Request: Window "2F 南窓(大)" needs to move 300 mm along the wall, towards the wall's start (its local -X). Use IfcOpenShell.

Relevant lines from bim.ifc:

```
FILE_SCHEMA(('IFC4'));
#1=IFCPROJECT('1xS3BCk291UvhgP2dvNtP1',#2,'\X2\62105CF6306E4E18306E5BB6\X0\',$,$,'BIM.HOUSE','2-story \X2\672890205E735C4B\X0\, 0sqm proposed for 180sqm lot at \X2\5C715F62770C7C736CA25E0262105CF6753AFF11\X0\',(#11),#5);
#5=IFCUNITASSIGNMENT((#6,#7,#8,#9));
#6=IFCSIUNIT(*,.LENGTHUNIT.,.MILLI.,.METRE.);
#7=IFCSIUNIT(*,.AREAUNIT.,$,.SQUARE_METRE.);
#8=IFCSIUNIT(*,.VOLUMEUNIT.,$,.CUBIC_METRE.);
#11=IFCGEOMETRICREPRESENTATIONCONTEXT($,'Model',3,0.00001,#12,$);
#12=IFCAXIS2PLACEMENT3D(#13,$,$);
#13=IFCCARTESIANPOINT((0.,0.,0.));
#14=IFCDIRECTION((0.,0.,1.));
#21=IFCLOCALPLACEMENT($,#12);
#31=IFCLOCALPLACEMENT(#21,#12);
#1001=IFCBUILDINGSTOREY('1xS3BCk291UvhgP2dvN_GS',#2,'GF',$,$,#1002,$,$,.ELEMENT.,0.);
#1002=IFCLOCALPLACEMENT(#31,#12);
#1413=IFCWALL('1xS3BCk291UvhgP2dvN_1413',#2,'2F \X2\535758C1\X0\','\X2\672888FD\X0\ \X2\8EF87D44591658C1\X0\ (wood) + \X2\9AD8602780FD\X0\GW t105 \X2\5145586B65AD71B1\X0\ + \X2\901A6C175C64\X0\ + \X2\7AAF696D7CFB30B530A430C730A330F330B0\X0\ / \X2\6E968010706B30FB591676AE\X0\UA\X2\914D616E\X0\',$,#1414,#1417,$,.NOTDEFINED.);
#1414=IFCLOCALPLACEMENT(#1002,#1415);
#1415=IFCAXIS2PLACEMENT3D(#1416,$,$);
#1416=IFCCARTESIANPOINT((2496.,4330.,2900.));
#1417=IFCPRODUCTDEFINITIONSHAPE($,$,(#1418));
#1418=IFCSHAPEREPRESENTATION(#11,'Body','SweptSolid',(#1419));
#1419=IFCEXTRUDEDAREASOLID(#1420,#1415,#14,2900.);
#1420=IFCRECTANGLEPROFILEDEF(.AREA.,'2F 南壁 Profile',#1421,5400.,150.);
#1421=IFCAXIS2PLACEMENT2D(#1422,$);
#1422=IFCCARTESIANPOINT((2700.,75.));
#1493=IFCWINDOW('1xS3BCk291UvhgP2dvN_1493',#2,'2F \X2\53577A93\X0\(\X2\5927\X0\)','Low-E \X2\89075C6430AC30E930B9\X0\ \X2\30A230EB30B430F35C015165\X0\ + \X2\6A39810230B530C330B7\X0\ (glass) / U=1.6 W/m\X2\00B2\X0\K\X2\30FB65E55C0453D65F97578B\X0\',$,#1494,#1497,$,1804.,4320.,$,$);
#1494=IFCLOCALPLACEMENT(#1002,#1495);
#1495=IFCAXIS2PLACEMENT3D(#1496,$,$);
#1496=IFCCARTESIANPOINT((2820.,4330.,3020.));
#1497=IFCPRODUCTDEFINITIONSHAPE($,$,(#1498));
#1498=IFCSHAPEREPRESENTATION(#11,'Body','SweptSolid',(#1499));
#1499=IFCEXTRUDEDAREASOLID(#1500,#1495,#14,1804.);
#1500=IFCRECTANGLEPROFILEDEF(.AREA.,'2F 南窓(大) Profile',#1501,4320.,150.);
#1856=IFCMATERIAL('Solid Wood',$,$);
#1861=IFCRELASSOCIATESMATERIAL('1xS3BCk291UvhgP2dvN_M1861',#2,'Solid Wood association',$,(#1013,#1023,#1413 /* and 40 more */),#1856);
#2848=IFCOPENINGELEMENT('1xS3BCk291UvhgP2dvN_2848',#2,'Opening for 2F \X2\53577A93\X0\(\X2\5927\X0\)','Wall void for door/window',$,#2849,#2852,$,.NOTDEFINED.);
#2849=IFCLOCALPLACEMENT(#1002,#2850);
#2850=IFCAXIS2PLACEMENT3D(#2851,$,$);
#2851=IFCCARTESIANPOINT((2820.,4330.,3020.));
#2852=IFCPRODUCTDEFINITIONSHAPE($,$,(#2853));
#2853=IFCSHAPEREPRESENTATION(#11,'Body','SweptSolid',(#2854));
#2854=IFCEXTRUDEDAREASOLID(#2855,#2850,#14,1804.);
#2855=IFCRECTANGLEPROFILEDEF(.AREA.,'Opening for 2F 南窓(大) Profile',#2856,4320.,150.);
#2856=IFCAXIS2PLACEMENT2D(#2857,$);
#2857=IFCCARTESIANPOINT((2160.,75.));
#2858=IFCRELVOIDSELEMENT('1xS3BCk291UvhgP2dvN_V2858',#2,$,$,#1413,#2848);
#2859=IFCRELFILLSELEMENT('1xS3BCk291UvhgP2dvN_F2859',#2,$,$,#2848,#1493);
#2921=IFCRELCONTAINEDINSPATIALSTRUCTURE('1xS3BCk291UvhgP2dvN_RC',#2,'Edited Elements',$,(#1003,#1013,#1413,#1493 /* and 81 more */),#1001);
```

```python
import ifcopenshell
import ifcopenshell.api.geometry
import ifcopenshell.util.placement

model = ifcopenshell.open("bim.ifc")

window = model.by_guid("1xS3BCk291UvhgP2dvN_1493")
opening = window.FillsVoids[0].RelatingOpeningElement
wall = opening.VoidsElements[0].RelatingBuildingElement

wall_matrix = ifcopenshell.util.placement.get_local_placement(wall.ObjectPlacement)
shift = wall_matrix[:3, 0] * -300.0
before = ifcopenshell.util.placement.get_local_placement(window.ObjectPlacement)[:3, 3].copy()

# The window is not placed relative to its opening, so move both.
for product in (opening, window):
    matrix = ifcopenshell.util.placement.get_local_placement(product.ObjectPlacement)
    matrix[:3, 3] += shift
    ifcopenshell.api.geometry.edit_object_placement(model, product=product, matrix=matrix, is_si=False)

after = ifcopenshell.util.placement.get_local_placement(window.ObjectPlacement)[:3, 3]
print("window moved by", (after - before).round(3) + 0.0)

model.write("bim_rev.ifc")
```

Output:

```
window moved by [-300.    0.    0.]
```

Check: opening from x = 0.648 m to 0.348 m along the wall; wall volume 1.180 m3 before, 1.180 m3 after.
